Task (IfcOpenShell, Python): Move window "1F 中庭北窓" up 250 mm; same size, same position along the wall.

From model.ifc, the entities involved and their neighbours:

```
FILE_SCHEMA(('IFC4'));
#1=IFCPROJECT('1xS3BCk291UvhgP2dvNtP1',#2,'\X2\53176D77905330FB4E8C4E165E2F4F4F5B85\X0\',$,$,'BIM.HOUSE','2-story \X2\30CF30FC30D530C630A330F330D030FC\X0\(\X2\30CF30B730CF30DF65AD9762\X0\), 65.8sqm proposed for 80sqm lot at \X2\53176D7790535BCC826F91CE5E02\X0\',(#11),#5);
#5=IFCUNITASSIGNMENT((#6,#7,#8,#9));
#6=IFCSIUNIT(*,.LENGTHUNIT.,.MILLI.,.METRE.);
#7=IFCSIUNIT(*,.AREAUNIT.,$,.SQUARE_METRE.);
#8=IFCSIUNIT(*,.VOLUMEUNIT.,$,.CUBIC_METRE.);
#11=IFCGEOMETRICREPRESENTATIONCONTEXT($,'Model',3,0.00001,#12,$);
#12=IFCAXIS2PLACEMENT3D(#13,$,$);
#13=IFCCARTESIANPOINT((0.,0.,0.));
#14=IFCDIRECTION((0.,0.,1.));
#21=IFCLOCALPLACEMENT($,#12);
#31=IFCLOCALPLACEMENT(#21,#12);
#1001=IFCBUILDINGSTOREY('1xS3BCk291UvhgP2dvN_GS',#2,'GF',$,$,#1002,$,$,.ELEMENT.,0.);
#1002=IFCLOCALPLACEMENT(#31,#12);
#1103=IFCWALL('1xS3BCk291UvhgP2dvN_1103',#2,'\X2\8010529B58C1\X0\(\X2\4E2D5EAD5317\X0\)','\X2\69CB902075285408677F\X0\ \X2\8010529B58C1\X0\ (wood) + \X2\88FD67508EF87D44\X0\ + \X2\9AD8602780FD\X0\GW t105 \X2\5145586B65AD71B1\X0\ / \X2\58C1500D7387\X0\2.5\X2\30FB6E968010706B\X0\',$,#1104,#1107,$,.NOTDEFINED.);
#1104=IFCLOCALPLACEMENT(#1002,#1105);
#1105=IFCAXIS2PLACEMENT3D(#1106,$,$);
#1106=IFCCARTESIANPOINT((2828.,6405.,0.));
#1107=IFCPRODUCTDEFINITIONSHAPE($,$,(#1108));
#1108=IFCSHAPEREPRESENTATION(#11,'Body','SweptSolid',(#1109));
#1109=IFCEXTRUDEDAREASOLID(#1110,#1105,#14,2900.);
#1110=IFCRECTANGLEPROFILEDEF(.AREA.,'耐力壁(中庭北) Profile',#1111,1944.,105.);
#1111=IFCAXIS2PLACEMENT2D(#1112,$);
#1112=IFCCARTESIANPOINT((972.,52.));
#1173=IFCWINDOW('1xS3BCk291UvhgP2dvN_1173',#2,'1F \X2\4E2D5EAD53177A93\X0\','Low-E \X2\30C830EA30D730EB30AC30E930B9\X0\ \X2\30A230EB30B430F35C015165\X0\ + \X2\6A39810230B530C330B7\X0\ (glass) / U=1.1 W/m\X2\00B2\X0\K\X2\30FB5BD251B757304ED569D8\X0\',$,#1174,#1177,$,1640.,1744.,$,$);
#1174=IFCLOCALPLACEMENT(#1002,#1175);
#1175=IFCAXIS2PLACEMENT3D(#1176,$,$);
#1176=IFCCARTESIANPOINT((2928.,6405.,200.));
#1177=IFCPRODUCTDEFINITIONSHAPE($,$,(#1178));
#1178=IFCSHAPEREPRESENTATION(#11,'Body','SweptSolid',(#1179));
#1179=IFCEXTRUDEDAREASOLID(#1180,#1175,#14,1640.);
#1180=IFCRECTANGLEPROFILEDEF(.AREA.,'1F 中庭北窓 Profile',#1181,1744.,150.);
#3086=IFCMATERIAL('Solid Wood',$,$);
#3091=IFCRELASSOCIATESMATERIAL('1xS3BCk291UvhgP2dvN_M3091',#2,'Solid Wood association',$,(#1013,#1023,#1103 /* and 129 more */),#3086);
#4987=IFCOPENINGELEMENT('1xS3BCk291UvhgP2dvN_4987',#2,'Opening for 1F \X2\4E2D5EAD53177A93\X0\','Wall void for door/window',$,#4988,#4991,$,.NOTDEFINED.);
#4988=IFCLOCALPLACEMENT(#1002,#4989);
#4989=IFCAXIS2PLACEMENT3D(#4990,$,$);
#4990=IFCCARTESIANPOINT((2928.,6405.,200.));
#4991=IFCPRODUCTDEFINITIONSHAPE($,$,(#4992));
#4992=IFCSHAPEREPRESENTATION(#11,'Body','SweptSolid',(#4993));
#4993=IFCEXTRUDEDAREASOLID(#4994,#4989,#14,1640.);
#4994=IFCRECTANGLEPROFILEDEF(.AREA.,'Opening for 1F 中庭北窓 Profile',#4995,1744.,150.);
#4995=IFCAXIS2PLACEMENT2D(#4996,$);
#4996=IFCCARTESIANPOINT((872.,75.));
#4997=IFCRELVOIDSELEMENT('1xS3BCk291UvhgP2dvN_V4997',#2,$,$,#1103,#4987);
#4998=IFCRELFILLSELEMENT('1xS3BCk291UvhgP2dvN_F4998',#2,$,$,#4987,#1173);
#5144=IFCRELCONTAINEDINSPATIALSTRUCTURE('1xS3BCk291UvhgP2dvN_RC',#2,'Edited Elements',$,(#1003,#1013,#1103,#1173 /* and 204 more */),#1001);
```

```python
import numpy as np
import ifcopenshell
import ifcopenshell.api.geometry
import ifcopenshell.util.placement
import ifcopenshell.util.unit

model = ifcopenshell.open("model.ifc")
unit_scale = ifcopenshell.util.unit.calculate_unit_scale(model)

window = model.by_guid("1xS3BCk291UvhgP2dvN_1173")
opening = window.FillsVoids[0].RelatingOpeningElement
dz = 0.25 / unit_scale

shift = np.array([0.0, 0.0, dz])
# The window is not placed relative to its opening, so move both.
for product in (opening, window):
    matrix = ifcopenshell.util.placement.get_local_placement(product.ObjectPlacement)
    matrix[:3, 3] += shift
    ifcopenshell.api.geometry.edit_object_placement(model, product=product, matrix=matrix, is_si=False)

print(f"moved by {dz * unit_scale:+.3f} m")

model.write("model_v2.ifc")
```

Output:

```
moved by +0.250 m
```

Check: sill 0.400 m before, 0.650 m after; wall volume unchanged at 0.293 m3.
